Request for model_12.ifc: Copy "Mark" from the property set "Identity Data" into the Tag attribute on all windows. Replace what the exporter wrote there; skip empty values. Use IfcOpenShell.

First a look at what the model holds.

```python
import ifcopenshell
import ifcopenshell.util.element

model = ifcopenshell.open("model_12.ifc")
print(model.schema)
windows = model.by_type("IfcWindow")
print(len(windows), "windows")
for e in windows[:8]:
    source = ifcopenshell.util.element.get_pset(e, "Identity Data", "Mark")
    target = e.Tag
    print(e.id(), repr(source), repr(target), sep=" | ")
```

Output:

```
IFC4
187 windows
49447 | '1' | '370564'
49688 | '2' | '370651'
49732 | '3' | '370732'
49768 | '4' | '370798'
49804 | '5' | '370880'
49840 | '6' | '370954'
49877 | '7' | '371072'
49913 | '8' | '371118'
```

```python
import ifcopenshell
import ifcopenshell.util.element

model = ifcopenshell.open("model_12.ifc")

count = 0
for e in model.by_type("IfcWindow"):
    value = ifcopenshell.util.element.get_pset(e, "Identity Data", "Mark")
    current = e.Tag
    if not value or not value.strip() or current == value:
        continue
    e.Tag = value
    count += 1

print(count, "windows updated")

model.write("model_12-out.ifc")
```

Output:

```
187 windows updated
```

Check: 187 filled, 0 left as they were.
